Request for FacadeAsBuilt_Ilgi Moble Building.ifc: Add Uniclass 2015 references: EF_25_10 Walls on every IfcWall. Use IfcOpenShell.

First a look at what the model holds.

```python
import ifcopenshell

model = ifcopenshell.open("FacadeAsBuilt_Ilgi Moble Building.ifc")
print(model.schema)
print("classifications:", [c.Name for c in model.by_type("IfcClassification")])
for ifc_class in ("IfcDoor", "IfcRoof", "IfcStair", "IfcWall", "IfcWindow"):
    print(ifc_class, len(model.by_type(ifc_class)))
```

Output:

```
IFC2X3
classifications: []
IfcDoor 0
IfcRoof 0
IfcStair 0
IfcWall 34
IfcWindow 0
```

```python
import ifcopenshell
import ifcopenshell.api.classification

model = ifcopenshell.open("FacadeAsBuilt_Ilgi Moble Building.ifc")

# IFC2X3 requires Source and Edition and has no link from the project to the system.
system = model.create_entity("IfcClassification", Source="NBS", Edition="2015", Name="Uniclass 2015")

codes = {
    "IfcWall": ("EF_25_10", "Walls"),
}
for ifc_class, (code, name) in codes.items():
    products = model.by_type(ifc_class)
    ifcopenshell.api.classification.add_reference(
        model, products=products, classification=system, identification=code, name=name
    )
    print(code, len(products))

model.write("FacadeAsBuilt_Ilgi Moble Building_edited.ifc")
```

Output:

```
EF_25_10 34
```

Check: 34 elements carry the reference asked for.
